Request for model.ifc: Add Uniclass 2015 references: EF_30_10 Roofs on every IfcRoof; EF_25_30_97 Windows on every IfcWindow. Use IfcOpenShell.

First a look at what the model holds.

```python
import ifcopenshell

model = ifcopenshell.open("model.ifc")
print(model.schema)
print("classifications:", [c.Name for c in model.by_type("IfcClassification")])
for ifc_class in ("IfcDoor", "IfcRoof", "IfcStair", "IfcWall", "IfcWindow"):
    print(ifc_class, len(model.by_type(ifc_class)))
```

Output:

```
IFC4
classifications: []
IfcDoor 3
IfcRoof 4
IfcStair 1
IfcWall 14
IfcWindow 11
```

```python
import ifcopenshell
import ifcopenshell.api.classification

model = ifcopenshell.open("model.ifc")

system = ifcopenshell.api.classification.add_classification(model, classification="Uniclass 2015")

codes = {
    "IfcRoof": ("EF_30_10", "Roofs"),
    "IfcWindow": ("EF_25_30_97", "Windows"),
}
for ifc_class, (code, name) in codes.items():
    products = model.by_type(ifc_class)
    ifcopenshell.api.classification.add_reference(
        model, products=products, classification=system, identification=code, name=name
    )
    print(code, len(products))

model.write("model_updated.ifc")
```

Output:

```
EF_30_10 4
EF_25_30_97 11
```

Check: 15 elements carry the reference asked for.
